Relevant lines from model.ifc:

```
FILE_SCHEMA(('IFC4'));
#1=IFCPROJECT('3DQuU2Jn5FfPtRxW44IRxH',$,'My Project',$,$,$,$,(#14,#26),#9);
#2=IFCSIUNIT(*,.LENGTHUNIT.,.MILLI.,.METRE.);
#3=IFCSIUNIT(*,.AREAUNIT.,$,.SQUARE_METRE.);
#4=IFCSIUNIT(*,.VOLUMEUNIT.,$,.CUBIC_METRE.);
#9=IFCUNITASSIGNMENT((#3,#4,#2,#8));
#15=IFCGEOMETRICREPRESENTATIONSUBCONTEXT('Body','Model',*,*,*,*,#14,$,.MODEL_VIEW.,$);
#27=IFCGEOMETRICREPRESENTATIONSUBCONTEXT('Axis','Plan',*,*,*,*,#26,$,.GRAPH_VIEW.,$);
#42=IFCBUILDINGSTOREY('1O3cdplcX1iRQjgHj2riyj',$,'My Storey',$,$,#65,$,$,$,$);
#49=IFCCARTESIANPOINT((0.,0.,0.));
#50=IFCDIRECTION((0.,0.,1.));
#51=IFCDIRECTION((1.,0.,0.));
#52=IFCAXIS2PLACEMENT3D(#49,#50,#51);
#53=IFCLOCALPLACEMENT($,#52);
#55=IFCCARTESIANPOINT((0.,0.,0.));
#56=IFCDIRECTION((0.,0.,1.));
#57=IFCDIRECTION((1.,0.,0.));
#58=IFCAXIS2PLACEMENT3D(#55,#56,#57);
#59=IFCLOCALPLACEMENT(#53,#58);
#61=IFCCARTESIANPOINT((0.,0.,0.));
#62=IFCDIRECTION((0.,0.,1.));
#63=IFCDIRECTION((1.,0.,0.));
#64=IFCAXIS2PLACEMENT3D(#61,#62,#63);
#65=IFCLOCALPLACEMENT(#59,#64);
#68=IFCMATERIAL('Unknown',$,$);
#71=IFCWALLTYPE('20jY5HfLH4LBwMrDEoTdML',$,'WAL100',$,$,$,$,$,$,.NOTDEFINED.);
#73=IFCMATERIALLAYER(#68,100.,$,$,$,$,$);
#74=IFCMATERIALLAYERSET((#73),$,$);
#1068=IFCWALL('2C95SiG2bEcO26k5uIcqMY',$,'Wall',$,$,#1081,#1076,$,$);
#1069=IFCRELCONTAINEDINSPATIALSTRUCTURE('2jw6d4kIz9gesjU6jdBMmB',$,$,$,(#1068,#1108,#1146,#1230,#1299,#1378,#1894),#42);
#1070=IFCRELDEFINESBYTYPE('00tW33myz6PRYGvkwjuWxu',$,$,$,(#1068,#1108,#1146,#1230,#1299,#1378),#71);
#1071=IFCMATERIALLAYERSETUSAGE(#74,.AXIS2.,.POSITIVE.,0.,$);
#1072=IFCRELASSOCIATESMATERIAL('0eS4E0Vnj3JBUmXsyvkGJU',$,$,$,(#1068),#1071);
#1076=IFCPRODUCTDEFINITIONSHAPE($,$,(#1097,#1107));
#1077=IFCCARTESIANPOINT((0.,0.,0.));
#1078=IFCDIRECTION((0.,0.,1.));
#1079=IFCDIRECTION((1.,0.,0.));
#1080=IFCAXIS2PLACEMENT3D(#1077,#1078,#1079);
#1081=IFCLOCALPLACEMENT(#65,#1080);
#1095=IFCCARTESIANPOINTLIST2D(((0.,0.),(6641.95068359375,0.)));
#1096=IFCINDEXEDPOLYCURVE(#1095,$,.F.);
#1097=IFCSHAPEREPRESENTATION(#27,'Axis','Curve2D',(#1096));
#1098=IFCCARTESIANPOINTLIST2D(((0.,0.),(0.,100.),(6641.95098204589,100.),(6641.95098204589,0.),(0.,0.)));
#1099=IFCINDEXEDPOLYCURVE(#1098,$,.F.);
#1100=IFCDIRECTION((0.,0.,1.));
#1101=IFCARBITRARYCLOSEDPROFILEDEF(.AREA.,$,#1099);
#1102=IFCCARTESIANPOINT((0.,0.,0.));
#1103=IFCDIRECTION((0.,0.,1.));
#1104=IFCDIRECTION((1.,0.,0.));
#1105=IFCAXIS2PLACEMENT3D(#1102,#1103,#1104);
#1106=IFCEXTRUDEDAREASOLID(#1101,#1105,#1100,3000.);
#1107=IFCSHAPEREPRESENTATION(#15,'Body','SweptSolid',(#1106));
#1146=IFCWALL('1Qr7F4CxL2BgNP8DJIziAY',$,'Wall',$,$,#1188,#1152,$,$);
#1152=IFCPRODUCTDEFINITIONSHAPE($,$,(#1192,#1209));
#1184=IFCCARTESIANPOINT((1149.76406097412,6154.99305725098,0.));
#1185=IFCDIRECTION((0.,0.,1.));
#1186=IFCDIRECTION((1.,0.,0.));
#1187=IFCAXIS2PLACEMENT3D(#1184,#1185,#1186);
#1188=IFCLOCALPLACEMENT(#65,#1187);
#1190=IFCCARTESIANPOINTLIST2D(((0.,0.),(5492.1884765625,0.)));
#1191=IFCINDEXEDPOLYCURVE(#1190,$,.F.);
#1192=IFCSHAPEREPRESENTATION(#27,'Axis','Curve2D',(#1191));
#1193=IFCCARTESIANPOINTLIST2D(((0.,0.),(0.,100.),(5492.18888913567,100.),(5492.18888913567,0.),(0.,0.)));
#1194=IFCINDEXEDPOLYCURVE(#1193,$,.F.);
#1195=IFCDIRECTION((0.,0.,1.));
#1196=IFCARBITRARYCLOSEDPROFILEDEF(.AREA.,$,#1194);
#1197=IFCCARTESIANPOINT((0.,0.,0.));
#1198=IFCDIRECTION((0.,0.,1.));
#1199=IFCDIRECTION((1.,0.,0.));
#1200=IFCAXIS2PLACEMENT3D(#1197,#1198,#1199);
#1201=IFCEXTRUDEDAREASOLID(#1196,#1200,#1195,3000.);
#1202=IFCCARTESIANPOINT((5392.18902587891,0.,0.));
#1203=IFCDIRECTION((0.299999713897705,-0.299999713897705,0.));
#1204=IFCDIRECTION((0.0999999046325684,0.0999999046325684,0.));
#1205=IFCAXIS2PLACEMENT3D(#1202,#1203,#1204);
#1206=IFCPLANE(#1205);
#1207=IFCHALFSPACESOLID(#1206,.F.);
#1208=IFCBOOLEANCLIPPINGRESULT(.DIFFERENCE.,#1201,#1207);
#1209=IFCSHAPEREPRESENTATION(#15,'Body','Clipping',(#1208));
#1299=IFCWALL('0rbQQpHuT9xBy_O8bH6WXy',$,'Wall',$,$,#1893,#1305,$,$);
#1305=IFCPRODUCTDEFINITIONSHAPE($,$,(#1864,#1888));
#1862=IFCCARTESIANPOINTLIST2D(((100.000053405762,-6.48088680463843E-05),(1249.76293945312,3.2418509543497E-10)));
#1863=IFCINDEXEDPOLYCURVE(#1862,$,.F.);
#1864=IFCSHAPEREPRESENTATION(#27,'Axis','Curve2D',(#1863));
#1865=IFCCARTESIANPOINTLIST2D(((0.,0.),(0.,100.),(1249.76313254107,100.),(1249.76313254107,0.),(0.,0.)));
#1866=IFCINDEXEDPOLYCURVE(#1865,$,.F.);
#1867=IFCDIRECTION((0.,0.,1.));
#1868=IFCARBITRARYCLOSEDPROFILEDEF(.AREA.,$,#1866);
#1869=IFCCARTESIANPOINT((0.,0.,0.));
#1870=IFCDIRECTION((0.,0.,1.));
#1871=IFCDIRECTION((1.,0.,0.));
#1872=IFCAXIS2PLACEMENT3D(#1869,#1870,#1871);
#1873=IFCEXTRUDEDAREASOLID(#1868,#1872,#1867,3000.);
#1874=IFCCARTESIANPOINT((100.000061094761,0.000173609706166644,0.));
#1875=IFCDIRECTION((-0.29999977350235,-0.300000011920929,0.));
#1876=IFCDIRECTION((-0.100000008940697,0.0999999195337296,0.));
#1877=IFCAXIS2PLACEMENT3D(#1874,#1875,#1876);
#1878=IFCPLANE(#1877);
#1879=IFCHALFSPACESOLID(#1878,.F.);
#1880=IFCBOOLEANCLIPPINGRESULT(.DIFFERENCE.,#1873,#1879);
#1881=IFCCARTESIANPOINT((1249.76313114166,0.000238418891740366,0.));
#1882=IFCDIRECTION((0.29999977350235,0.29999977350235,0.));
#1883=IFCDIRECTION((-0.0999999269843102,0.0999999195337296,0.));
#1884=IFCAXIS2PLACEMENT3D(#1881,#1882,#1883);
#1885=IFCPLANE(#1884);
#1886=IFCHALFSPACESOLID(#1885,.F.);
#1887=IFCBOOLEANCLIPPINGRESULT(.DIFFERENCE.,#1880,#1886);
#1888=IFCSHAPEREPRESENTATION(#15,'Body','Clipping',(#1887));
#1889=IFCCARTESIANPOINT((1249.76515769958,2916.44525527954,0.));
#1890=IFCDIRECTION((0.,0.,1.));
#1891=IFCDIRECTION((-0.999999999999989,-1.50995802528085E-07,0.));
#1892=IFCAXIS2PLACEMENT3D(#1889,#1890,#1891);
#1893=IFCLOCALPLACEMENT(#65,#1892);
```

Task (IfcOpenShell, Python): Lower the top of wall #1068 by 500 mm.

```python
import ifcopenshell
import ifcopenshell.geom
import ifcopenshell.util.representation
import ifcopenshell.util.shape

model = ifcopenshell.open("model.ifc")
settings = ifcopenshell.geom.settings()


def volume(element):
    """Net volume in cubic metres, openings subtracted."""
    shape = ifcopenshell.geom.create_shape(settings, element)
    return ifcopenshell.util.shape.get_volume(shape.geometry)


wall = model.by_guid("2C95SiG2bEcO26k5uIcqMY")
before = volume(wall)

body = ifcopenshell.util.representation.get_representation(wall, "Model", "Body")
solid = body.Items[0]
old_height = solid.Depth
solid.Depth -= 500.0
after = volume(wall)

print(f"height {old_height:g} -> {solid.Depth:g}, volume {before:.3f} -> {after:.3f} m3")

model.write("model_rev.ifc")
```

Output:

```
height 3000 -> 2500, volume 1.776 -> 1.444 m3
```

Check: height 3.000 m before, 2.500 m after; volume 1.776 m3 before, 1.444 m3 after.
